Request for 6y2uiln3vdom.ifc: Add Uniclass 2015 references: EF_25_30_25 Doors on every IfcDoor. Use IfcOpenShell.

First a look at what the model holds.

```python
import ifcopenshell

model = ifcopenshell.open("6y2uiln3vdom.ifc")
print(model.schema)
print("classifications:", [c.Name for c in model.by_type("IfcClassification")])
for ifc_class in ("IfcDoor", "IfcRoof", "IfcStair", "IfcWall", "IfcWindow"):
    print(ifc_class, len(model.by_type(ifc_class)))
```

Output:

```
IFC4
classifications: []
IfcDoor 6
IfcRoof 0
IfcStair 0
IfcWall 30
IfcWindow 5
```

```python
import ifcopenshell
import ifcopenshell.api.classification

model = ifcopenshell.open("6y2uiln3vdom.ifc")

system = ifcopenshell.api.classification.add_classification(model, classification="Uniclass 2015")

codes = {
    "IfcDoor": ("EF_25_30_25", "Doors"),
}
for ifc_class, (code, name) in codes.items():
    products = model.by_type(ifc_class)
    ifcopenshell.api.classification.add_reference(
        model, products=products, classification=system, identification=code, name=name
    )
    print(code, len(products))

model.write("6y2uiln3vdom_v2.ifc")
```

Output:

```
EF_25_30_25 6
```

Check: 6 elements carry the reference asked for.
